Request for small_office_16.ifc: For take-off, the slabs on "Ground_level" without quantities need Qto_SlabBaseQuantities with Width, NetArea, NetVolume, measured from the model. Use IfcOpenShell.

First a look at what the model holds.

```python
import ifcopenshell
import ifcopenshell.util.element
import ifcopenshell.util.unit

model = ifcopenshell.open("small_office_16.ifc")
print(model.schema)
for unit_type in ("LENGTHUNIT", "AREAUNIT", "VOLUMEUNIT"):
    print(unit_type, ifcopenshell.util.unit.calculate_unit_scale(model, unit_type))
storey = next(s for s in model.by_type("IfcBuildingStorey") if s.Name == "Ground_level")
slabs = [e for e in ifcopenshell.util.element.get_decomposition(storey) if e.is_a("IfcSlab")]
for e in sorted(slabs, key=lambda e: e.id()):
    print(e.id(), e.is_a(), e.Name, list(ifcopenshell.util.element.get_psets(e, qtos_only=True)), sep=" | ")
```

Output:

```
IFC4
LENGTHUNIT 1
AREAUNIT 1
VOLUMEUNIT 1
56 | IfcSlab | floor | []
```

```python
import ifcopenshell
import ifcopenshell.api.pset
import ifcopenshell.geom
import ifcopenshell.util.element
import ifcopenshell.util.shape
import ifcopenshell.util.unit

model = ifcopenshell.open("small_office_16.ifc")
unit_scale = ifcopenshell.util.unit.calculate_unit_scale(model)
area_scale = ifcopenshell.util.unit.calculate_unit_scale(model, "AREAUNIT")
volume_scale = ifcopenshell.util.unit.calculate_unit_scale(model, "VOLUMEUNIT")
settings = ifcopenshell.geom.settings()

storey = next(s for s in model.by_type("IfcBuildingStorey") if s.Name == "Ground_level")
slabs = [e for e in ifcopenshell.util.element.get_decomposition(storey) if e.is_a("IfcSlab")]

for e in sorted(slabs, key=lambda e: e.id()):
    if ifcopenshell.util.element.get_psets(e, qtos_only=True, should_inherit=False):
        continue
    # Geometry comes back in metres, in the element's own axes.
    shape = ifcopenshell.geom.create_shape(settings, e)
    values = {
        "Width": ifcopenshell.util.shape.get_z(shape.geometry) / unit_scale,
        "NetArea": ifcopenshell.util.shape.get_footprint_area(shape.geometry) / area_scale,
        "NetVolume": ifcopenshell.util.shape.get_volume(shape.geometry) / volume_scale,
    }
    qto = ifcopenshell.api.pset.add_qto(model, product=e, name="Qto_SlabBaseQuantities")
    ifcopenshell.api.pset.edit_qto(model, qto=qto, properties=values)
    print(e.id(), {k: round(v, 3) for k, v in values.items()})

model.write("small_office_16-out.ifc")
```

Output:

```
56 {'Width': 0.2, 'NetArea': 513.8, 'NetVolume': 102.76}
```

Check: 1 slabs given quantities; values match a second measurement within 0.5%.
